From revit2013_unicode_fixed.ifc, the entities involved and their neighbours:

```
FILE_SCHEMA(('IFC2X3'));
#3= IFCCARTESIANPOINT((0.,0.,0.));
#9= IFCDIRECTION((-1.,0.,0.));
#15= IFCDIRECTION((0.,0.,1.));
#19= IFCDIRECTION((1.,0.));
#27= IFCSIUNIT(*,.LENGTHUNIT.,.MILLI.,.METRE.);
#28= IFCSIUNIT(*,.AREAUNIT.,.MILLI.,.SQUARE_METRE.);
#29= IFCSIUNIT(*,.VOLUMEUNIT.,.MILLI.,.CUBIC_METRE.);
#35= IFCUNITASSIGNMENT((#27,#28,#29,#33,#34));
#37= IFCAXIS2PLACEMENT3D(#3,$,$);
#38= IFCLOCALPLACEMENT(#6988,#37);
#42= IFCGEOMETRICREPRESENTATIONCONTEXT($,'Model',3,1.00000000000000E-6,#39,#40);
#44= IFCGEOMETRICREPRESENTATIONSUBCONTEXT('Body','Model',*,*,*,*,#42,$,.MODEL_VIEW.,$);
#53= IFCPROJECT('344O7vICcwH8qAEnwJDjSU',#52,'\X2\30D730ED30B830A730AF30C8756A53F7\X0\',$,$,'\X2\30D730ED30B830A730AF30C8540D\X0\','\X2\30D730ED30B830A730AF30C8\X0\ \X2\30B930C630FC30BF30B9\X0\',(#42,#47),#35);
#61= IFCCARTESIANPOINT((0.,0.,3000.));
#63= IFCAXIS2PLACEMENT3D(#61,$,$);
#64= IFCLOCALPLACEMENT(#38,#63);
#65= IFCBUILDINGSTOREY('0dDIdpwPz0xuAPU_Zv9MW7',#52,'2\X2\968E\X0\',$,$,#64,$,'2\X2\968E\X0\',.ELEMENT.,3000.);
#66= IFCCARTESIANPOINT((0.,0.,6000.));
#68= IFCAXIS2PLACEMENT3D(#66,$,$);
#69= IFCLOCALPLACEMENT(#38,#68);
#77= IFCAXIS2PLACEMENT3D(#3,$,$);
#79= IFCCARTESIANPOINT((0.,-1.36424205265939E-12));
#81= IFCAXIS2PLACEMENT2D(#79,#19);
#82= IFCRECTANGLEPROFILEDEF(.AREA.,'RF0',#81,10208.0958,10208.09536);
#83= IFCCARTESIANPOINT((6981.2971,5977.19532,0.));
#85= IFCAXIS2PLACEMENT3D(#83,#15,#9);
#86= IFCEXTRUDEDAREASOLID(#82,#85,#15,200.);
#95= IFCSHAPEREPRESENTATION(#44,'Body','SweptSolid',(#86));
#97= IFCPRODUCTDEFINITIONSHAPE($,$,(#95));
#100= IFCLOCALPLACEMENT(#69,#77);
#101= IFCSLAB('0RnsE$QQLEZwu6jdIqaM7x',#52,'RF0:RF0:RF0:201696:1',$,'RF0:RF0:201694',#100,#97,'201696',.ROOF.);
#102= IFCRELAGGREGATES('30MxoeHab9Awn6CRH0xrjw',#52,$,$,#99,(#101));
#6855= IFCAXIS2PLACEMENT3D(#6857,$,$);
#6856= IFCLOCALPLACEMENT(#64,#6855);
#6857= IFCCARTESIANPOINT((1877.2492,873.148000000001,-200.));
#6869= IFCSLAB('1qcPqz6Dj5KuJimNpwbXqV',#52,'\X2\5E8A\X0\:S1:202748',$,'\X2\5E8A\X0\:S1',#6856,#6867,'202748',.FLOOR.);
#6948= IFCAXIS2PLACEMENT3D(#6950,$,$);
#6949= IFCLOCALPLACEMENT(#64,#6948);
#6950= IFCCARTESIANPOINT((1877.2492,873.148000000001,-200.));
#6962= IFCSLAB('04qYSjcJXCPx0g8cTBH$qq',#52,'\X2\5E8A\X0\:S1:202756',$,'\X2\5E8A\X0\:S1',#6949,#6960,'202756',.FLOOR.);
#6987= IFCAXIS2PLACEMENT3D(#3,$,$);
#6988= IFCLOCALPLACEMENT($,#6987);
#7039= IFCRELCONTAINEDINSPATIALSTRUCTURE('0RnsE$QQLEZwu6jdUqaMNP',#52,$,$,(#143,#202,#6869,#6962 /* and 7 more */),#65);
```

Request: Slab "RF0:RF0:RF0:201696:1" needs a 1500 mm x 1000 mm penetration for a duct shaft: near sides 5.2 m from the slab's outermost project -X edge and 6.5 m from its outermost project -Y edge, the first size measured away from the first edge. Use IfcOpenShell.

```python
import numpy as np
import ifcopenshell
import ifcopenshell.api.feature
import ifcopenshell.api.geometry
import ifcopenshell.api.root
import ifcopenshell.geom
import ifcopenshell.util.placement
import ifcopenshell.util.representation
import ifcopenshell.util.shape
import ifcopenshell.util.unit

model = ifcopenshell.open("revit2013_unicode_fixed.ifc")
unit_scale = ifcopenshell.util.unit.calculate_unit_scale(model)
settings = ifcopenshell.geom.settings()


def volume(element):
    """Net volume in cubic metres, openings subtracted."""
    shape = ifcopenshell.geom.create_shape(settings, element)
    return ifcopenshell.util.shape.get_volume(shape.geometry)


slab = model.by_guid("0RnsE$QQLEZwu6jdIqaM7x")
before = volume(slab)

# Extent in the slab's own axes, in metres. The edges named are its -X and -Y sides.
slab_shape = ifcopenshell.geom.create_shape(settings, slab)
vertices = ifcopenshell.util.shape.get_vertices(slab_shape.geometry)
x_min, y_min, bottom = vertices.min(axis=0)
top = vertices[:, 2].max()

opening = ifcopenshell.api.root.create_entity(model, ifc_class="IfcOpeningElement", name="Duct shaft opening")
context = ifcopenshell.util.representation.get_context(model, "Model", "Body", "MODEL_VIEW")
width, depth = 1.5, 1
outline = [(0.0, 0.0), (width, 0.0), (width, depth), (0.0, depth), (0.0, 0.0)]
# Overshoot both faces by 50 mm so the cut is clean.
shape = ifcopenshell.api.geometry.add_slab_representation(
    model, context=context, depth=top - bottom + 0.1, polyline=outline
)
ifcopenshell.api.geometry.assign_representation(model, product=opening, representation=shape)

matrix = ifcopenshell.util.placement.get_local_placement(slab.ObjectPlacement)
matrix[:, 3] = matrix @ np.append(np.array([x_min + 5.2, y_min + 6.5, bottom - 0.05]) / unit_scale, 1.0)
ifcopenshell.api.geometry.edit_object_placement(model, product=opening, matrix=matrix, is_si=False)
ifcopenshell.api.feature.add_feature(model, feature=opening, element=slab)

after = volume(slab)

print(f"slab volume {before:.3f} -> {after:.3f} m3")

model.write("revit2013_unicode_fixed_edited.ifc")
```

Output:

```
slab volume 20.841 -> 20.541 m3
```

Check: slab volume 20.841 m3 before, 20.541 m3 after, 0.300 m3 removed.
